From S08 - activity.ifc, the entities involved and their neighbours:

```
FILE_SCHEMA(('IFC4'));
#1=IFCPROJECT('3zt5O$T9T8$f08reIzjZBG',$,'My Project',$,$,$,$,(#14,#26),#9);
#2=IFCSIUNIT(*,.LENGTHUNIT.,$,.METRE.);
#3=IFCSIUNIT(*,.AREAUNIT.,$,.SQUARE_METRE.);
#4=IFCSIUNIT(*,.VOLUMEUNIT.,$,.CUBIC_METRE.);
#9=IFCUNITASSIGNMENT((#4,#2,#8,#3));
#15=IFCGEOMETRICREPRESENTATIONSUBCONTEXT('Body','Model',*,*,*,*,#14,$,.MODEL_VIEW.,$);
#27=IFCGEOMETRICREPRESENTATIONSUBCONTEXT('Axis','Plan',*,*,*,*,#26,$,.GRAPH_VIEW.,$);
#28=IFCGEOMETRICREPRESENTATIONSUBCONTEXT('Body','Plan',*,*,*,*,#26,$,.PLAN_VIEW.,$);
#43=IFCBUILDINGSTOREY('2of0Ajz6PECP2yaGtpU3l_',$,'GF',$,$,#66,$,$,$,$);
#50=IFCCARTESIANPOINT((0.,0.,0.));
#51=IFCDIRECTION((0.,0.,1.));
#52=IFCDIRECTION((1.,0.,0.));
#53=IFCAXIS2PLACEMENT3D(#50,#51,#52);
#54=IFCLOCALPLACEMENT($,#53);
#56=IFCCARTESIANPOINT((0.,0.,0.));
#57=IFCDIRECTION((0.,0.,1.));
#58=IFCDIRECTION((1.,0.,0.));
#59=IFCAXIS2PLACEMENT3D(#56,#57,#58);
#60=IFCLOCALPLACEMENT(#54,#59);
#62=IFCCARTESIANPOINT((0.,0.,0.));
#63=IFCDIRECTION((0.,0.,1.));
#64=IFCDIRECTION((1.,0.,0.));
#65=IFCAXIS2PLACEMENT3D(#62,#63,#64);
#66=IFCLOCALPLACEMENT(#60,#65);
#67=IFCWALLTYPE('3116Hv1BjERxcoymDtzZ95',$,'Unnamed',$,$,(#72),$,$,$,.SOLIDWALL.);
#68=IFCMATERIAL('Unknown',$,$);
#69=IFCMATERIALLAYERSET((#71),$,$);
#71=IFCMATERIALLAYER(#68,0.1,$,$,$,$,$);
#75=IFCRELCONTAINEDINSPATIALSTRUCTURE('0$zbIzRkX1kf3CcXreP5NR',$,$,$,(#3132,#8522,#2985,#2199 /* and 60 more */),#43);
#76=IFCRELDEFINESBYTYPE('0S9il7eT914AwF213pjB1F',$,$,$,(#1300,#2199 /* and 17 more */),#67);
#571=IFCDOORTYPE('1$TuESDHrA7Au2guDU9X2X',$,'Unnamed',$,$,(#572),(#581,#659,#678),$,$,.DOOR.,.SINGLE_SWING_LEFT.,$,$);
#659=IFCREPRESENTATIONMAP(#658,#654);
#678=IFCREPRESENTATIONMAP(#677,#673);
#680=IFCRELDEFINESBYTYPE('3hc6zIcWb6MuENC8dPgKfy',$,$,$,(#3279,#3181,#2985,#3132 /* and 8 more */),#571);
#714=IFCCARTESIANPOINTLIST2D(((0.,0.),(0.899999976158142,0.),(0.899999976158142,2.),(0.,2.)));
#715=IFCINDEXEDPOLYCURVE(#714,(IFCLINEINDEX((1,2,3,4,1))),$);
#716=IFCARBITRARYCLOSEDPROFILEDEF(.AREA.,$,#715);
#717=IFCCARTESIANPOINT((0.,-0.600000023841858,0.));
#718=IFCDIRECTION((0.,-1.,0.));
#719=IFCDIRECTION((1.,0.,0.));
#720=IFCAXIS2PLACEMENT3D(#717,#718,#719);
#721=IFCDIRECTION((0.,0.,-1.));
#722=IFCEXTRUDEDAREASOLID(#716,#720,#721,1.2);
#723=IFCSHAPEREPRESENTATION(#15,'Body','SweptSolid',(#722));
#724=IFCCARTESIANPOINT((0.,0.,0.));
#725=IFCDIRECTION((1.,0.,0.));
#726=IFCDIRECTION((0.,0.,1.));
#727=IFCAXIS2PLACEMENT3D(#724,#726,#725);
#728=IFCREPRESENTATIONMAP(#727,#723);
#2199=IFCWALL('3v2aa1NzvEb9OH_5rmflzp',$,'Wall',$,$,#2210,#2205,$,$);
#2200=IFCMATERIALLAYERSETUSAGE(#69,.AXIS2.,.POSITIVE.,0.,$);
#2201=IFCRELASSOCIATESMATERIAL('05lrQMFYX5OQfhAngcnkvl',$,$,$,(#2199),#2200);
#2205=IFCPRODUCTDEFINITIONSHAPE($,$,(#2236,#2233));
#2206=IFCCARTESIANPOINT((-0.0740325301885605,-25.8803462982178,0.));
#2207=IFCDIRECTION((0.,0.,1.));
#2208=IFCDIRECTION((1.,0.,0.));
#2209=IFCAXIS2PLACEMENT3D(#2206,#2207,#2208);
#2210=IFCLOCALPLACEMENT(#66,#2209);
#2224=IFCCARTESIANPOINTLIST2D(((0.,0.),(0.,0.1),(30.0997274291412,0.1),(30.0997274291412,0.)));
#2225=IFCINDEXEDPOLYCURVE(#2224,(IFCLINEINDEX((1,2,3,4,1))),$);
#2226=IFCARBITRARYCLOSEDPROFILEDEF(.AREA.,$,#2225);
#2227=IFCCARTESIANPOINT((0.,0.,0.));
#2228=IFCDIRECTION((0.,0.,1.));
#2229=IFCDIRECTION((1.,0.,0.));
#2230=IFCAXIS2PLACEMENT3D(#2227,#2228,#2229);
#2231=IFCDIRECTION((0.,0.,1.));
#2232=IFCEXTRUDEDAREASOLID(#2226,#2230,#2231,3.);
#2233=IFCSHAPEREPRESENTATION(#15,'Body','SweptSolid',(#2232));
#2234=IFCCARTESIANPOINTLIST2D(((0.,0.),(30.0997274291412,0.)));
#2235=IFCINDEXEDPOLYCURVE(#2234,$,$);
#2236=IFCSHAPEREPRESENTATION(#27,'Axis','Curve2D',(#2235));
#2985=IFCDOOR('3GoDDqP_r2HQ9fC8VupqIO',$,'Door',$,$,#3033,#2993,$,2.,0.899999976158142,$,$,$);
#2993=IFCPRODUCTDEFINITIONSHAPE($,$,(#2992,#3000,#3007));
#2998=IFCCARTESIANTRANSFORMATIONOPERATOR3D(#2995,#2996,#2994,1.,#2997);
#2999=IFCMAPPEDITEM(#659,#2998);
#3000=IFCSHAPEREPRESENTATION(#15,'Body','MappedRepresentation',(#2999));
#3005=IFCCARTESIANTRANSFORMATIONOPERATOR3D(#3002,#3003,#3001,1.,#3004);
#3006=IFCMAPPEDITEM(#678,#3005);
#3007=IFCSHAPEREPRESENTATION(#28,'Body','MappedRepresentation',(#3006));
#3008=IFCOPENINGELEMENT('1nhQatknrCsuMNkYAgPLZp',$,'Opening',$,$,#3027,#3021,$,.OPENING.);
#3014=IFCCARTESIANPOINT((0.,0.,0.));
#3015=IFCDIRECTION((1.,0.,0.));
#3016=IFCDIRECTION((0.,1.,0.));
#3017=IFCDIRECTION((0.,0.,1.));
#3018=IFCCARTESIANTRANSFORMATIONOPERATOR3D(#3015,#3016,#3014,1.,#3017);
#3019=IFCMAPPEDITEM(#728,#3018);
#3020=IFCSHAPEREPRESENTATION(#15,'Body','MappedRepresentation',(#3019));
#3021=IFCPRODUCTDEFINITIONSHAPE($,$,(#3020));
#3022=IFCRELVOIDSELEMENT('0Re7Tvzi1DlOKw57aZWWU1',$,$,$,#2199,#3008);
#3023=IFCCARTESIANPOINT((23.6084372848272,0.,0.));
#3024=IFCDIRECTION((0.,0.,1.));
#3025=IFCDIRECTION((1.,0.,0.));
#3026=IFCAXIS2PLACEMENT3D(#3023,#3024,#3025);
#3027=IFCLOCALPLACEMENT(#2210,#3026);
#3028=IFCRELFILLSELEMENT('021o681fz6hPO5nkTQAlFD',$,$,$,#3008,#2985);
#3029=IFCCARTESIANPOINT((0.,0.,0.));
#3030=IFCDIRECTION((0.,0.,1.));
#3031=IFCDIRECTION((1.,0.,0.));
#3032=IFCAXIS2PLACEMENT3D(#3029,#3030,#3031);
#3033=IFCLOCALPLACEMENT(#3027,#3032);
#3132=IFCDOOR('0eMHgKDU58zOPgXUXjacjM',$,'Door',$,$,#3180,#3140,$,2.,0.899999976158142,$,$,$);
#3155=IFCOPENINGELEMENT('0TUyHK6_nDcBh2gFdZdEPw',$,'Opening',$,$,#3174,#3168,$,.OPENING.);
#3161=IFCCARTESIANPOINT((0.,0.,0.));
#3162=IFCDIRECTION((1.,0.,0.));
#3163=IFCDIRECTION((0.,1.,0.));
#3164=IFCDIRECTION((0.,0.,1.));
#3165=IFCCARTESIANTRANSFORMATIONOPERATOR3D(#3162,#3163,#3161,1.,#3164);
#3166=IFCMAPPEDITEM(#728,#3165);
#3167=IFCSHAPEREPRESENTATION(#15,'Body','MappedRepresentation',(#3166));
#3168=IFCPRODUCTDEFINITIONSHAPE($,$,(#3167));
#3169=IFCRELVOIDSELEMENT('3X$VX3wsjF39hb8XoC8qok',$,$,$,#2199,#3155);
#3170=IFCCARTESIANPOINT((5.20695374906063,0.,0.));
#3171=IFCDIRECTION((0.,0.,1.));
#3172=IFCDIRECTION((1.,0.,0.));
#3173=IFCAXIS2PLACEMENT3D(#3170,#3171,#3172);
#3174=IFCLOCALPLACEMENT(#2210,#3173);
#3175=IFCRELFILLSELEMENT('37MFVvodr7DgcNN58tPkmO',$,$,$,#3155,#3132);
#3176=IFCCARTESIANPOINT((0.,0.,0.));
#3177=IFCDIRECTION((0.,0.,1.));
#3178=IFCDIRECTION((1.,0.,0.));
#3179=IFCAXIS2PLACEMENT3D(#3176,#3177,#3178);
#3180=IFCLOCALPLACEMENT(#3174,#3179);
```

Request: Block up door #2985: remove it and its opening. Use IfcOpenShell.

```python
import ifcopenshell
import ifcopenshell.api.feature
import ifcopenshell.api.root
import ifcopenshell.geom
import ifcopenshell.util.shape

model = ifcopenshell.open("S08 - activity.ifc")
settings = ifcopenshell.geom.settings()


def volume(element):
    """Net volume in cubic metres, openings subtracted."""
    shape = ifcopenshell.geom.create_shape(settings, element)
    return ifcopenshell.util.shape.get_volume(shape.geometry)


door = model.by_guid("3GoDDqP_r2HQ9fC8VupqIO")
opening = door.FillsVoids[0].RelatingOpeningElement
wall = opening.VoidsElements[0].RelatingBuildingElement
before = volume(wall)

ifcopenshell.api.root.remove_product(model, product=door)
ifcopenshell.api.feature.remove_feature(model, feature=opening)

after = volume(wall)

print(f"wall volume {before:.3f} -> {after:.3f} m3")

model.write("S08 - activity_v2.ifc")
```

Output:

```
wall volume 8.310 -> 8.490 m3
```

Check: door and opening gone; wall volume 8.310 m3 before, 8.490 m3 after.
